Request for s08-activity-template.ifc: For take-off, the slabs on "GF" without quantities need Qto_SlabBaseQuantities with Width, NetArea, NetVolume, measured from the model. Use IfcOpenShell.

First a look at what the model holds.

```python
import ifcopenshell
import ifcopenshell.util.element
import ifcopenshell.util.unit

model = ifcopenshell.open("s08-activity-template.ifc")
print(model.schema)
for unit_type in ("LENGTHUNIT", "AREAUNIT", "VOLUMEUNIT"):
    print(unit_type, ifcopenshell.util.unit.calculate_unit_scale(model, unit_type))
storey = next(s for s in model.by_type("IfcBuildingStorey") if s.Name == "GF")
slabs = [e for e in ifcopenshell.util.element.get_decomposition(storey) if e.is_a("IfcSlab")]
for e in sorted(slabs, key=lambda e: e.id()):
    print(e.id(), e.is_a(), e.Name, list(ifcopenshell.util.element.get_psets(e, qtos_only=True)), sep=" | ")
```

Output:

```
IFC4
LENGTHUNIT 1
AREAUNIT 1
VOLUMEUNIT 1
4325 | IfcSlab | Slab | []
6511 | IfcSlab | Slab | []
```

```python
import ifcopenshell
import ifcopenshell.api.pset
import ifcopenshell.geom
import ifcopenshell.util.element
import ifcopenshell.util.shape
import ifcopenshell.util.unit

model = ifcopenshell.open("s08-activity-template.ifc")
unit_scale = ifcopenshell.util.unit.calculate_unit_scale(model)
area_scale = ifcopenshell.util.unit.calculate_unit_scale(model, "AREAUNIT")
volume_scale = ifcopenshell.util.unit.calculate_unit_scale(model, "VOLUMEUNIT")
settings = ifcopenshell.geom.settings()

storey = next(s for s in model.by_type("IfcBuildingStorey") if s.Name == "GF")
slabs = [e for e in ifcopenshell.util.element.get_decomposition(storey) if e.is_a("IfcSlab")]

for e in sorted(slabs, key=lambda e: e.id()):
    if ifcopenshell.util.element.get_psets(e, qtos_only=True, should_inherit=False):
        continue
    # Geometry comes back in metres, in the element's own axes.
    shape = ifcopenshell.geom.create_shape(settings, e)
    values = {
        "Width": ifcopenshell.util.shape.get_z(shape.geometry) / unit_scale,
        "NetArea": ifcopenshell.util.shape.get_footprint_area(shape.geometry) / area_scale,
        "NetVolume": ifcopenshell.util.shape.get_volume(shape.geometry) / volume_scale,
    }
    qto = ifcopenshell.api.pset.add_qto(model, product=e, name="Qto_SlabBaseQuantities")
    ifcopenshell.api.pset.edit_qto(model, qto=qto, properties=values)
    print(e.id(), {k: round(v, 3) for k, v in values.items()})

model.write("s08-activity-template_rev.ifc")
```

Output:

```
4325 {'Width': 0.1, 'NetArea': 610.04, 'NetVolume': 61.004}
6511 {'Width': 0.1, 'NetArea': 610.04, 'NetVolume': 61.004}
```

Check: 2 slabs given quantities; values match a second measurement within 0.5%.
